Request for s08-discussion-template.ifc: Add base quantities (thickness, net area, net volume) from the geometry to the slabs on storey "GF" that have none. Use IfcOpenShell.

First a look at what the model holds.

```python
import ifcopenshell
import ifcopenshell.util.element
import ifcopenshell.util.unit

model = ifcopenshell.open("s08-discussion-template.ifc")
print(model.schema)
for unit_type in ("LENGTHUNIT", "AREAUNIT", "VOLUMEUNIT"):
    print(unit_type, ifcopenshell.util.unit.calculate_unit_scale(model, unit_type))
storey = next(s for s in model.by_type("IfcBuildingStorey") if s.Name == "GF")
slabs = [e for e in ifcopenshell.util.element.get_decomposition(storey) if e.is_a("IfcSlab")]
for e in sorted(slabs, key=lambda e: e.id()):
    print(e.id(), e.is_a(), e.Name, list(ifcopenshell.util.element.get_psets(e, qtos_only=True)), sep=" | ")
```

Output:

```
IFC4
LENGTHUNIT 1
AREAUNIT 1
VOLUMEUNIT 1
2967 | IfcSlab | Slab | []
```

```python
import ifcopenshell
import ifcopenshell.api.pset
import ifcopenshell.geom
import ifcopenshell.util.element
import ifcopenshell.util.shape
import ifcopenshell.util.unit

model = ifcopenshell.open("s08-discussion-template.ifc")
unit_scale = ifcopenshell.util.unit.calculate_unit_scale(model)
area_scale = ifcopenshell.util.unit.calculate_unit_scale(model, "AREAUNIT")
volume_scale = ifcopenshell.util.unit.calculate_unit_scale(model, "VOLUMEUNIT")
settings = ifcopenshell.geom.settings()

storey = next(s for s in model.by_type("IfcBuildingStorey") if s.Name == "GF")
slabs = [e for e in ifcopenshell.util.element.get_decomposition(storey) if e.is_a("IfcSlab")]

for e in sorted(slabs, key=lambda e: e.id()):
    if ifcopenshell.util.element.get_psets(e, qtos_only=True, should_inherit=False):
        continue
    # Geometry comes back in metres, in the element's own axes.
    shape = ifcopenshell.geom.create_shape(settings, e)
    values = {
        "Width": ifcopenshell.util.shape.get_z(shape.geometry) / unit_scale,
        "NetArea": ifcopenshell.util.shape.get_footprint_area(shape.geometry) / area_scale,
        "NetVolume": ifcopenshell.util.shape.get_volume(shape.geometry) / volume_scale,
    }
    qto = ifcopenshell.api.pset.add_qto(model, product=e, name="Qto_SlabBaseQuantities")
    ifcopenshell.api.pset.edit_qto(model, qto=qto, properties=values)
    print(e.id(), {k: round(v, 3) for k, v in values.items()})

model.write("s08-discussion-template_updated.ifc")
```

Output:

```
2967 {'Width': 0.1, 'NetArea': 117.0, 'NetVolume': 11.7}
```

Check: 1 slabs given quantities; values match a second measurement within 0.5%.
